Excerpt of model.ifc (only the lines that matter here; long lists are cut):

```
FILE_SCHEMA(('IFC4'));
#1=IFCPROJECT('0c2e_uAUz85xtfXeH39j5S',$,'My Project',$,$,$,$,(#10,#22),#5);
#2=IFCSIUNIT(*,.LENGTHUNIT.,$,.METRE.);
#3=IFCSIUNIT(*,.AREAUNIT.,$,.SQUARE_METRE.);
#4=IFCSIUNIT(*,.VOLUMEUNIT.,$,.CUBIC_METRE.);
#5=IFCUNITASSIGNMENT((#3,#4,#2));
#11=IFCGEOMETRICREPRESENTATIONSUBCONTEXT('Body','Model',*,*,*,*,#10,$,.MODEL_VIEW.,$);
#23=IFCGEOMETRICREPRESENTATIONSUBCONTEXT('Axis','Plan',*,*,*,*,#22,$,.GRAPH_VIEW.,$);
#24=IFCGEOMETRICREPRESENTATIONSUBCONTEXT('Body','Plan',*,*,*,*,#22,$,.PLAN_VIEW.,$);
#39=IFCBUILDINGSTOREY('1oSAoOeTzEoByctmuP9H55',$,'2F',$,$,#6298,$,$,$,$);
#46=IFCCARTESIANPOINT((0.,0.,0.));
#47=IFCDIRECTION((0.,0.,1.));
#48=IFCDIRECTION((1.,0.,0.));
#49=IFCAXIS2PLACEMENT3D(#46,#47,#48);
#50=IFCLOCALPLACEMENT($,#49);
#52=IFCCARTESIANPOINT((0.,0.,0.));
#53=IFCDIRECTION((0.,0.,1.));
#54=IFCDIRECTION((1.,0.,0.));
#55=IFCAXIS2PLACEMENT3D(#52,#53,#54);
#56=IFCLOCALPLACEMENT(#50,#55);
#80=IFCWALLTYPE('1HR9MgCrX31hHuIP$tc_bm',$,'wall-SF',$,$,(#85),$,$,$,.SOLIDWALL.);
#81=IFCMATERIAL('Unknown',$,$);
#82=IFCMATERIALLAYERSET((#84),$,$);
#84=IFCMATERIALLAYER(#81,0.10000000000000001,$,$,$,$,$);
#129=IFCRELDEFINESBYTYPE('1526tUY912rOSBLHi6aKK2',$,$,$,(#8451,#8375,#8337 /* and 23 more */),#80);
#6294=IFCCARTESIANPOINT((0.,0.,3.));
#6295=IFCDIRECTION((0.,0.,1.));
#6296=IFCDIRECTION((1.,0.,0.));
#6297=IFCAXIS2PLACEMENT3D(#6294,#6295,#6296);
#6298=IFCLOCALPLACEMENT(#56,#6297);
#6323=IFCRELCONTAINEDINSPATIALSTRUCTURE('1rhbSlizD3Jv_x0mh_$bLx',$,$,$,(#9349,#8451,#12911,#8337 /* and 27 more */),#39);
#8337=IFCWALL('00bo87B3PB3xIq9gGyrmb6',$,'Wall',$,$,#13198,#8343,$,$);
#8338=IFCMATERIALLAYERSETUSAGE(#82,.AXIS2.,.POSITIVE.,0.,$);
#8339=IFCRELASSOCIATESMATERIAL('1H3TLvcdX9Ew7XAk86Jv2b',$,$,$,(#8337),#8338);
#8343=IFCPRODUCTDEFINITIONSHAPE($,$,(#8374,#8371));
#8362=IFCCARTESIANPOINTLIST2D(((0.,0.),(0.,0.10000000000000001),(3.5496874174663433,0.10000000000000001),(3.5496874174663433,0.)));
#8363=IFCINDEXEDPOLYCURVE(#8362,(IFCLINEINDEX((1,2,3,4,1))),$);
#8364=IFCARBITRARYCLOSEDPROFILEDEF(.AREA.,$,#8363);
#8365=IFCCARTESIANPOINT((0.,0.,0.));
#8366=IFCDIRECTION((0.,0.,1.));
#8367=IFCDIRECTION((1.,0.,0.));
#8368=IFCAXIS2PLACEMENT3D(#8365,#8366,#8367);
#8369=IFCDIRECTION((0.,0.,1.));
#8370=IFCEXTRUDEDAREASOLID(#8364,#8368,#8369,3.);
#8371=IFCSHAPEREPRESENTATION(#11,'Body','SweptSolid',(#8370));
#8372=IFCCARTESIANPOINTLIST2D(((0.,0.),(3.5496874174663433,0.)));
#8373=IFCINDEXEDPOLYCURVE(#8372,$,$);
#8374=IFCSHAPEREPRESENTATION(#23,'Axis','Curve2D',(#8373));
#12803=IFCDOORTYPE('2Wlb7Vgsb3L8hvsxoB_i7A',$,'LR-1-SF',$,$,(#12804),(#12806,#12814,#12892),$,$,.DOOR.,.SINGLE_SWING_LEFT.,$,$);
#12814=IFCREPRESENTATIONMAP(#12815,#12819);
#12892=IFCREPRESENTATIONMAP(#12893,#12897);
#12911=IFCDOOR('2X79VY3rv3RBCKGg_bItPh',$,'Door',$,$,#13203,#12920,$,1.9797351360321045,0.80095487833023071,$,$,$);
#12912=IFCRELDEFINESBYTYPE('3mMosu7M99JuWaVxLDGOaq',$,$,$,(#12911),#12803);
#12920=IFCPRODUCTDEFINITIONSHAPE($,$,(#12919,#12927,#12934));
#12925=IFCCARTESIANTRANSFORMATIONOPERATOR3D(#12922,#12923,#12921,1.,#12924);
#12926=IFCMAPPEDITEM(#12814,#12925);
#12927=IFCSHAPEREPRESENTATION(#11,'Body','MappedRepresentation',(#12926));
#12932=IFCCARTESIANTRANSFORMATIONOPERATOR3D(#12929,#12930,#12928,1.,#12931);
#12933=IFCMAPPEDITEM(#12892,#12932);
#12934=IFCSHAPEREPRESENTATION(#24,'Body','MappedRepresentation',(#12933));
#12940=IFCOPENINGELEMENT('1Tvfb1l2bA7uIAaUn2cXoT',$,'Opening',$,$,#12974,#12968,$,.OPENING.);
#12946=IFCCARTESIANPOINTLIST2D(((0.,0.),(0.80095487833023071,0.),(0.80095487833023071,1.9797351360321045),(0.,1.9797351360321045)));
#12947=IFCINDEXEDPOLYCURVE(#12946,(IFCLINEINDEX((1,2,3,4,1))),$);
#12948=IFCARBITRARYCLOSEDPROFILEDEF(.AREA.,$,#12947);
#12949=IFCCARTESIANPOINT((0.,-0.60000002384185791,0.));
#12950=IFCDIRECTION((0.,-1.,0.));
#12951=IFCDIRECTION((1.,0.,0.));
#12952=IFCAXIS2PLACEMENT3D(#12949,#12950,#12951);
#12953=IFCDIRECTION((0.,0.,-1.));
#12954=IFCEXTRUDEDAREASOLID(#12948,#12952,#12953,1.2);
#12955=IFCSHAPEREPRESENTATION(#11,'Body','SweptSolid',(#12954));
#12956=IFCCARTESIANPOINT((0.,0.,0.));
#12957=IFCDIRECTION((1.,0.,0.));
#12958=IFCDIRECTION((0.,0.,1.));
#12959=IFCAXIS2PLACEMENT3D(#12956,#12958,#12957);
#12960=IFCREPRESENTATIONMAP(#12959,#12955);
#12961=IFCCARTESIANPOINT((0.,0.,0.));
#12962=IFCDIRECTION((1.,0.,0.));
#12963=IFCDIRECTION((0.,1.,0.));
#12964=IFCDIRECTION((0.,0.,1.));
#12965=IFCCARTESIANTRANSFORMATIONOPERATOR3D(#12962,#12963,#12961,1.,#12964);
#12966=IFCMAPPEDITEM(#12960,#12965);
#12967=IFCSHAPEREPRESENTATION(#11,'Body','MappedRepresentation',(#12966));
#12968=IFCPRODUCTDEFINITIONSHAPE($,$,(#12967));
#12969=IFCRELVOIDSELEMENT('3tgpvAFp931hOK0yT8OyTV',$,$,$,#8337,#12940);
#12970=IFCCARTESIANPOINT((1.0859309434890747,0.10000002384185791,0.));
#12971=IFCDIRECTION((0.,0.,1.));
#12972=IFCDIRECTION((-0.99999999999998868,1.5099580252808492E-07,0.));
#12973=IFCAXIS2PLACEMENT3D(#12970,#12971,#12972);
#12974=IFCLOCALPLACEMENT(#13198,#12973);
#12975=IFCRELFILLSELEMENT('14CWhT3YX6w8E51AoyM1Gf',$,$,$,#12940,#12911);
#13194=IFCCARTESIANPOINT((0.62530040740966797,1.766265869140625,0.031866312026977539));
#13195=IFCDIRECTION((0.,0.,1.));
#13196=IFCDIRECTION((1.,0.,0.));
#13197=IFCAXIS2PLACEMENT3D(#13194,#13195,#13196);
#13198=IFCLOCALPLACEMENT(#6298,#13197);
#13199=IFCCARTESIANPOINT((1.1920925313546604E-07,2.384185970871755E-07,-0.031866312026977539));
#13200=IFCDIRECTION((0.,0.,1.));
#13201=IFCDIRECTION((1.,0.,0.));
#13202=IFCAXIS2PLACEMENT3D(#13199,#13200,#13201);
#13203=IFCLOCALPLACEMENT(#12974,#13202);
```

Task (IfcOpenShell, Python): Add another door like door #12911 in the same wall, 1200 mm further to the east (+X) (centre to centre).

```python
import ifcopenshell
import ifcopenshell.api.feature
import ifcopenshell.api.geometry
import ifcopenshell.api.root
import ifcopenshell.geom
import ifcopenshell.util.element
import ifcopenshell.util.placement
import ifcopenshell.util.shape

model = ifcopenshell.open("model.ifc")
settings = ifcopenshell.geom.settings()


def volume(element):
    """Net volume in cubic metres, openings subtracted."""
    shape = ifcopenshell.geom.create_shape(settings, element)
    return ifcopenshell.util.shape.get_volume(shape.geometry)


door = model.by_guid("2X79VY3rv3RBCKGg_bItPh")
opening = door.FillsVoids[0].RelatingOpeningElement
wall = opening.VoidsElements[0].RelatingBuildingElement
before = volume(wall)
shift = ifcopenshell.util.placement.get_local_placement(wall.ObjectPlacement)[:3, 0] * 1.2

# copy_class copies the void relationship, type, container and properties, but no geometry.
new_opening = ifcopenshell.api.root.copy_class(model, product=opening)
new_opening.Representation = ifcopenshell.util.element.copy_deep(
    model, opening.Representation, exclude=["IfcGeometricRepresentationContext", "IfcRepresentationMap"]
)
new_door = ifcopenshell.api.root.copy_class(model, product=door)
new_door.Representation = ifcopenshell.util.element.copy_deep(
    model, door.Representation, exclude=["IfcGeometricRepresentationContext", "IfcRepresentationMap"]
)
ifcopenshell.api.feature.add_filling(model, opening=new_opening, element=new_door)

for old, new in ((opening, new_opening), (door, new_door)):
    matrix = ifcopenshell.util.placement.get_local_placement(old.ObjectPlacement)
    matrix[:3, 3] += shift
    ifcopenshell.api.geometry.edit_object_placement(model, product=new, matrix=matrix, is_si=False)

after = volume(wall)

print(f"wall volume {before:.3f} -> {after:.3f} m3")

model.write("model_rev.ifc")
```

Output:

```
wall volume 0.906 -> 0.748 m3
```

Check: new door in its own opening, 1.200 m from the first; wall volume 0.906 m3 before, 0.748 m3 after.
